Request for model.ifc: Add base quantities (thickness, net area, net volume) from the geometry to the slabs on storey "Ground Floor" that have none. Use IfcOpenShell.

First a look at what the model holds.

```python
import ifcopenshell
import ifcopenshell.util.element
import ifcopenshell.util.unit

model = ifcopenshell.open("model.ifc")
print(model.schema)
for unit_type in ("LENGTHUNIT", "AREAUNIT", "VOLUMEUNIT"):
    print(unit_type, ifcopenshell.util.unit.calculate_unit_scale(model, unit_type))
storey = next(s for s in model.by_type("IfcBuildingStorey") if s.Name == "Ground Floor")
slabs = [e for e in ifcopenshell.util.element.get_decomposition(storey) if e.is_a("IfcSlab")]
for e in sorted(slabs, key=lambda e: e.id()):
    print(e.id(), e.is_a(), e.Name, list(ifcopenshell.util.element.get_psets(e, qtos_only=True)), sep=" | ")
```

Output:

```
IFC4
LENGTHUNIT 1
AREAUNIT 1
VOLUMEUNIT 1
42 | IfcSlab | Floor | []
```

```python
import ifcopenshell
import ifcopenshell.api.pset
import ifcopenshell.geom
import ifcopenshell.util.element
import ifcopenshell.util.shape
import ifcopenshell.util.unit

model = ifcopenshell.open("model.ifc")
unit_scale = ifcopenshell.util.unit.calculate_unit_scale(model)
area_scale = ifcopenshell.util.unit.calculate_unit_scale(model, "AREAUNIT")
volume_scale = ifcopenshell.util.unit.calculate_unit_scale(model, "VOLUMEUNIT")
settings = ifcopenshell.geom.settings()

storey = next(s for s in model.by_type("IfcBuildingStorey") if s.Name == "Ground Floor")
slabs = [e for e in ifcopenshell.util.element.get_decomposition(storey) if e.is_a("IfcSlab")]

for e in sorted(slabs, key=lambda e: e.id()):
    if ifcopenshell.util.element.get_psets(e, qtos_only=True, should_inherit=False):
        continue
    # Geometry comes back in metres, in the element's own axes.
    shape = ifcopenshell.geom.create_shape(settings, e)
    values = {
        "Width": ifcopenshell.util.shape.get_z(shape.geometry) / unit_scale,
        "NetArea": ifcopenshell.util.shape.get_footprint_area(shape.geometry) / area_scale,
        "NetVolume": ifcopenshell.util.shape.get_volume(shape.geometry) / volume_scale,
    }
    qto = ifcopenshell.api.pset.add_qto(model, product=e, name="Qto_SlabBaseQuantities")
    ifcopenshell.api.pset.edit_qto(model, qto=qto, properties=values)
    print(e.id(), {k: round(v, 3) for k, v in values.items()})

model.write("model_v2.ifc")
```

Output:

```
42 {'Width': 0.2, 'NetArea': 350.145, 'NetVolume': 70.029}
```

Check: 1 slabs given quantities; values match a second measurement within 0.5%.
